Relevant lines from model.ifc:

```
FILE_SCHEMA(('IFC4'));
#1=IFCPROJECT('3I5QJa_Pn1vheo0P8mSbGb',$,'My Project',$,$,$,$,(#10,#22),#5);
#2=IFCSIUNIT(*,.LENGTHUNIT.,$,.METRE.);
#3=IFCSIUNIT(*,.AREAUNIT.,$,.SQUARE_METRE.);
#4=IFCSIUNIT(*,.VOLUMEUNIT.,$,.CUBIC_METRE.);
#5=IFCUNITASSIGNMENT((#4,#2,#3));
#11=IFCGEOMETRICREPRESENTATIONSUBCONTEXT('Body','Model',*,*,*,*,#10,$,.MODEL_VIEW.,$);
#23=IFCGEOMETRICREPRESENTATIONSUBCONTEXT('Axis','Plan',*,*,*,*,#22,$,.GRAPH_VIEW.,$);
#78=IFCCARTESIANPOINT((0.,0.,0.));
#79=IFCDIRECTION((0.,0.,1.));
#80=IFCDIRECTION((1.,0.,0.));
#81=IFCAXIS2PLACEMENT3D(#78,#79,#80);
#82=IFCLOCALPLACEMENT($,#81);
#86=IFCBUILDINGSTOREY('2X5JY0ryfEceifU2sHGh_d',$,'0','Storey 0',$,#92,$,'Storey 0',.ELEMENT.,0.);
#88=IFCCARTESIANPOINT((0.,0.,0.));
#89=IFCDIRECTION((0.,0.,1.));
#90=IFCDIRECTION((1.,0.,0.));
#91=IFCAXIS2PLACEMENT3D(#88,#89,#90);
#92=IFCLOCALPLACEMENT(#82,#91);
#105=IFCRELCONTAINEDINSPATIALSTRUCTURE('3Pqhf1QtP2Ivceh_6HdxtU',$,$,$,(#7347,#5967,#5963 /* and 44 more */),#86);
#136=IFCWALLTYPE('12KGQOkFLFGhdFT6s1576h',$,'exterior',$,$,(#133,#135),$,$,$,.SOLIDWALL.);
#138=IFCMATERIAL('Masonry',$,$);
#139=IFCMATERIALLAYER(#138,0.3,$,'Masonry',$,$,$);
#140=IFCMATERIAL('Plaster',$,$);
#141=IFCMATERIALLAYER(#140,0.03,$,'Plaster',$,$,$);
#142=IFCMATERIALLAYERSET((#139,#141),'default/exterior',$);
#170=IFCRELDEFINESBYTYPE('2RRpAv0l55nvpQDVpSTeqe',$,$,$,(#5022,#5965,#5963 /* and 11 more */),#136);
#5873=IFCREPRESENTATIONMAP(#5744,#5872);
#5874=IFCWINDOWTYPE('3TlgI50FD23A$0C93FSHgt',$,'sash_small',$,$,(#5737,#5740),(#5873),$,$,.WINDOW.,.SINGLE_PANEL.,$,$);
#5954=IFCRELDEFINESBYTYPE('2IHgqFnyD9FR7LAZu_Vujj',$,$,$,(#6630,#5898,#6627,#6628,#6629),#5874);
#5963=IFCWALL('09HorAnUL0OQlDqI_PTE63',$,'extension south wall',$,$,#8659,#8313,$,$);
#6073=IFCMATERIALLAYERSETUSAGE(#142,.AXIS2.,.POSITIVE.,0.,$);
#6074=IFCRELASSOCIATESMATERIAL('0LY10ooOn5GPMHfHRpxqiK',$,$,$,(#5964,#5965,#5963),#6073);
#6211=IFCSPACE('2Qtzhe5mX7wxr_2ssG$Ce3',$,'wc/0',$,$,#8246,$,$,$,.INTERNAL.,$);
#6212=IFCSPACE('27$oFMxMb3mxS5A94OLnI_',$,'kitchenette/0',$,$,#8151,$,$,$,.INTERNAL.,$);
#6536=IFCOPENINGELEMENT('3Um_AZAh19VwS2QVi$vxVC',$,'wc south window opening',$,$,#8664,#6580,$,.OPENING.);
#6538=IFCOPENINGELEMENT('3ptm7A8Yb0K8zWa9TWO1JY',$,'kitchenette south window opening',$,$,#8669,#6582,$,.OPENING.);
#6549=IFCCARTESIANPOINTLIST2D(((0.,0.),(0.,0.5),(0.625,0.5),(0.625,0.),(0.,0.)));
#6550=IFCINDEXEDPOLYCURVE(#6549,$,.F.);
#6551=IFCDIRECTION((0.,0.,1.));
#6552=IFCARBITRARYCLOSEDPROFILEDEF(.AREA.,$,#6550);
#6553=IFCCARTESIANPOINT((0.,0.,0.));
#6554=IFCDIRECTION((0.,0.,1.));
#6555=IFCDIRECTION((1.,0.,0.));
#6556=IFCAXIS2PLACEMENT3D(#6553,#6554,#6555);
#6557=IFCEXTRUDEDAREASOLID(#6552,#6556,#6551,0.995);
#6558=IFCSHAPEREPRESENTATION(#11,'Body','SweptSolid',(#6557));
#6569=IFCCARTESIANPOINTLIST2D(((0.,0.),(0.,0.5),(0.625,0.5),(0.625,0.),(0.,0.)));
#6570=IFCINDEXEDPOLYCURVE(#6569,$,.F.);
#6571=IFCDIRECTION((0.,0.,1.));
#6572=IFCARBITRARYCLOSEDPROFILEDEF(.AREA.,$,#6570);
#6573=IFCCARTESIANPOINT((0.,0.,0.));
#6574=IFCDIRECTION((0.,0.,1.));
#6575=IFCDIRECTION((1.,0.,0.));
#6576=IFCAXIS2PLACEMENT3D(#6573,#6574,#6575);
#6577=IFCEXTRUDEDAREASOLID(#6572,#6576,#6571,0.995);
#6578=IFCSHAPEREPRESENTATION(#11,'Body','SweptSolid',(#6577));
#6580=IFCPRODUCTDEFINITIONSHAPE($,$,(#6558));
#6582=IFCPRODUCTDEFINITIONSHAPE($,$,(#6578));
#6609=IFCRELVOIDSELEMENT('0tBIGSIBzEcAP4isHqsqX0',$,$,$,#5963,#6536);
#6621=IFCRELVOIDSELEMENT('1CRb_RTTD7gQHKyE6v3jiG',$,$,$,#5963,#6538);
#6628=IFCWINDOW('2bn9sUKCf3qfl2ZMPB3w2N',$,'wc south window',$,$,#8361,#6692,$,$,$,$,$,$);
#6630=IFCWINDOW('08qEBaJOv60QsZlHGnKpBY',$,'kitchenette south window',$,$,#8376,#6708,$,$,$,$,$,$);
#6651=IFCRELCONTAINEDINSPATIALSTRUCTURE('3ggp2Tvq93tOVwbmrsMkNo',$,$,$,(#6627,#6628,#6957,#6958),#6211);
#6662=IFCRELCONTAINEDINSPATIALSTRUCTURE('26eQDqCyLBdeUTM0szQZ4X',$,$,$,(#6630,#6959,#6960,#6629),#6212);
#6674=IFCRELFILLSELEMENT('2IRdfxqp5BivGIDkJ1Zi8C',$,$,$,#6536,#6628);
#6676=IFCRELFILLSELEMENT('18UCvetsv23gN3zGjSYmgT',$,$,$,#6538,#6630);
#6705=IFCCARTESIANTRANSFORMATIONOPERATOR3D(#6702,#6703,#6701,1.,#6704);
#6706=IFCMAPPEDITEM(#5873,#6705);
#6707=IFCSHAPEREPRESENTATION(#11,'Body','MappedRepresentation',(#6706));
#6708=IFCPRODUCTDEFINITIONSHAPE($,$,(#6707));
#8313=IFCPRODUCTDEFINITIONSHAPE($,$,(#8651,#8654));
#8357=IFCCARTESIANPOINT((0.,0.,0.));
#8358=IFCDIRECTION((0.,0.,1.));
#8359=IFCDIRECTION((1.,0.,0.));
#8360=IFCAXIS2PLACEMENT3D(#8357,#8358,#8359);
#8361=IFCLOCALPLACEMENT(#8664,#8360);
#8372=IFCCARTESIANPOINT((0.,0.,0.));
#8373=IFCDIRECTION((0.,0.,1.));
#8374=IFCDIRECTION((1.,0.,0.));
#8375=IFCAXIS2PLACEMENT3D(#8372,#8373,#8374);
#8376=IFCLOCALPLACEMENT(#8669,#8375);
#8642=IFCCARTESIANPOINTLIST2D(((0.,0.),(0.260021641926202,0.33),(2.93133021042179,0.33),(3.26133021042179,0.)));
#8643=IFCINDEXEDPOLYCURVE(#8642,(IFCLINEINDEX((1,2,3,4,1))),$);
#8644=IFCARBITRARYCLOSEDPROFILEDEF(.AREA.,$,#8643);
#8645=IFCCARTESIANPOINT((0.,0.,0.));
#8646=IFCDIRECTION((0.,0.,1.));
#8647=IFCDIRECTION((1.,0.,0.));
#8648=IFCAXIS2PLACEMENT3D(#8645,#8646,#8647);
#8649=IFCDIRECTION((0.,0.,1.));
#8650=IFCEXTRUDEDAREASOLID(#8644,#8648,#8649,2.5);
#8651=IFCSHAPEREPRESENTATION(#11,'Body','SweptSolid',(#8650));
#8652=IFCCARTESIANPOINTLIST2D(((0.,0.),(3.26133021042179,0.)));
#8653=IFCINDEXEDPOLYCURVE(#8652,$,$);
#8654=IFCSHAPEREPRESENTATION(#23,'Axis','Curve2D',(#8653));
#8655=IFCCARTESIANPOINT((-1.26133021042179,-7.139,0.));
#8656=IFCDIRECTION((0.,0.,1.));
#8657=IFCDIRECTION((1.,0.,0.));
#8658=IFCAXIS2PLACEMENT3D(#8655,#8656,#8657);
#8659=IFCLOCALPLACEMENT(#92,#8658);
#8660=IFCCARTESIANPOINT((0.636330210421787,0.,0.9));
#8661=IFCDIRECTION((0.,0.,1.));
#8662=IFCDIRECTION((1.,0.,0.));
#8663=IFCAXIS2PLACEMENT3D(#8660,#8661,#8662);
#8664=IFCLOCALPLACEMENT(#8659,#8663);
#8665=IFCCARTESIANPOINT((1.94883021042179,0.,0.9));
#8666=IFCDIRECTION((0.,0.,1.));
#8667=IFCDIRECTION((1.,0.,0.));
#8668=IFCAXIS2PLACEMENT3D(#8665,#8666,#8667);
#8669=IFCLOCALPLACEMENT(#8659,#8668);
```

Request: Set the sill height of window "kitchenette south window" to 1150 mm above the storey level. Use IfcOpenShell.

```python
import numpy as np
import ifcopenshell
import ifcopenshell.api.geometry
import ifcopenshell.geom
import ifcopenshell.util.element
import ifcopenshell.util.placement
import ifcopenshell.util.shape
import ifcopenshell.util.unit

model = ifcopenshell.open("model.ifc")
unit_scale = ifcopenshell.util.unit.calculate_unit_scale(model)

window = model.by_guid("08qEBaJOv60QsZlHGnKpBY")
opening = window.FillsVoids[0].RelatingOpeningElement
storey = ifcopenshell.util.element.get_container(window, ifc_class="IfcBuildingStorey")
level = ifcopenshell.util.placement.get_local_placement(storey.ObjectPlacement)[2, 3]

# The opening's origin need not be at the sill, so measure its lowest point.
shape = ifcopenshell.geom.create_shape(ifcopenshell.geom.settings(), opening)
bottom = ifcopenshell.util.shape.get_shape_bottom_elevation(shape, shape.geometry) / unit_scale
dz = level + 1.15 / unit_scale - bottom

shift = np.array([0.0, 0.0, dz])
# The window is placed relative to its opening, so it follows when the opening moves.
matrix = ifcopenshell.util.placement.get_local_placement(opening.ObjectPlacement)
matrix[:3, 3] += shift
ifcopenshell.api.geometry.edit_object_placement(
    model, product=opening, matrix=matrix, is_si=False, should_transform_children=True
)

print(f"moved by {dz * unit_scale:+.3f} m")

model.write("model_rev.ifc")
```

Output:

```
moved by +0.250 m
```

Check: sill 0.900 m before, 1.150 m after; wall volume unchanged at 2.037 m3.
